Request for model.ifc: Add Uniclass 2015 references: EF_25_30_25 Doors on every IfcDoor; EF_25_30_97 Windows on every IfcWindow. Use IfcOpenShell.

First a look at what the model holds.

```python
import ifcopenshell

model = ifcopenshell.open("model.ifc")
print(model.schema)
print("classifications:", [c.Name for c in model.by_type("IfcClassification")])
for ifc_class in ("IfcDoor", "IfcRoof", "IfcStair", "IfcWall", "IfcWindow"):
    print(ifc_class, len(model.by_type(ifc_class)))
```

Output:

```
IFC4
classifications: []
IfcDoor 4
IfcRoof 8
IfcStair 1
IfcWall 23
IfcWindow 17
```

```python
import ifcopenshell
import ifcopenshell.api.classification

model = ifcopenshell.open("model.ifc")

system = ifcopenshell.api.classification.add_classification(model, classification="Uniclass 2015")

codes = {
    "IfcDoor": ("EF_25_30_25", "Doors"),
    "IfcWindow": ("EF_25_30_97", "Windows"),
}
for ifc_class, (code, name) in codes.items():
    products = model.by_type(ifc_class)
    ifcopenshell.api.classification.add_reference(
        model, products=products, classification=system, identification=code, name=name
    )
    print(code, len(products))

model.write("model_rev.ifc")
```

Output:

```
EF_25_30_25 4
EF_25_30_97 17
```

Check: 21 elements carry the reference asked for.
